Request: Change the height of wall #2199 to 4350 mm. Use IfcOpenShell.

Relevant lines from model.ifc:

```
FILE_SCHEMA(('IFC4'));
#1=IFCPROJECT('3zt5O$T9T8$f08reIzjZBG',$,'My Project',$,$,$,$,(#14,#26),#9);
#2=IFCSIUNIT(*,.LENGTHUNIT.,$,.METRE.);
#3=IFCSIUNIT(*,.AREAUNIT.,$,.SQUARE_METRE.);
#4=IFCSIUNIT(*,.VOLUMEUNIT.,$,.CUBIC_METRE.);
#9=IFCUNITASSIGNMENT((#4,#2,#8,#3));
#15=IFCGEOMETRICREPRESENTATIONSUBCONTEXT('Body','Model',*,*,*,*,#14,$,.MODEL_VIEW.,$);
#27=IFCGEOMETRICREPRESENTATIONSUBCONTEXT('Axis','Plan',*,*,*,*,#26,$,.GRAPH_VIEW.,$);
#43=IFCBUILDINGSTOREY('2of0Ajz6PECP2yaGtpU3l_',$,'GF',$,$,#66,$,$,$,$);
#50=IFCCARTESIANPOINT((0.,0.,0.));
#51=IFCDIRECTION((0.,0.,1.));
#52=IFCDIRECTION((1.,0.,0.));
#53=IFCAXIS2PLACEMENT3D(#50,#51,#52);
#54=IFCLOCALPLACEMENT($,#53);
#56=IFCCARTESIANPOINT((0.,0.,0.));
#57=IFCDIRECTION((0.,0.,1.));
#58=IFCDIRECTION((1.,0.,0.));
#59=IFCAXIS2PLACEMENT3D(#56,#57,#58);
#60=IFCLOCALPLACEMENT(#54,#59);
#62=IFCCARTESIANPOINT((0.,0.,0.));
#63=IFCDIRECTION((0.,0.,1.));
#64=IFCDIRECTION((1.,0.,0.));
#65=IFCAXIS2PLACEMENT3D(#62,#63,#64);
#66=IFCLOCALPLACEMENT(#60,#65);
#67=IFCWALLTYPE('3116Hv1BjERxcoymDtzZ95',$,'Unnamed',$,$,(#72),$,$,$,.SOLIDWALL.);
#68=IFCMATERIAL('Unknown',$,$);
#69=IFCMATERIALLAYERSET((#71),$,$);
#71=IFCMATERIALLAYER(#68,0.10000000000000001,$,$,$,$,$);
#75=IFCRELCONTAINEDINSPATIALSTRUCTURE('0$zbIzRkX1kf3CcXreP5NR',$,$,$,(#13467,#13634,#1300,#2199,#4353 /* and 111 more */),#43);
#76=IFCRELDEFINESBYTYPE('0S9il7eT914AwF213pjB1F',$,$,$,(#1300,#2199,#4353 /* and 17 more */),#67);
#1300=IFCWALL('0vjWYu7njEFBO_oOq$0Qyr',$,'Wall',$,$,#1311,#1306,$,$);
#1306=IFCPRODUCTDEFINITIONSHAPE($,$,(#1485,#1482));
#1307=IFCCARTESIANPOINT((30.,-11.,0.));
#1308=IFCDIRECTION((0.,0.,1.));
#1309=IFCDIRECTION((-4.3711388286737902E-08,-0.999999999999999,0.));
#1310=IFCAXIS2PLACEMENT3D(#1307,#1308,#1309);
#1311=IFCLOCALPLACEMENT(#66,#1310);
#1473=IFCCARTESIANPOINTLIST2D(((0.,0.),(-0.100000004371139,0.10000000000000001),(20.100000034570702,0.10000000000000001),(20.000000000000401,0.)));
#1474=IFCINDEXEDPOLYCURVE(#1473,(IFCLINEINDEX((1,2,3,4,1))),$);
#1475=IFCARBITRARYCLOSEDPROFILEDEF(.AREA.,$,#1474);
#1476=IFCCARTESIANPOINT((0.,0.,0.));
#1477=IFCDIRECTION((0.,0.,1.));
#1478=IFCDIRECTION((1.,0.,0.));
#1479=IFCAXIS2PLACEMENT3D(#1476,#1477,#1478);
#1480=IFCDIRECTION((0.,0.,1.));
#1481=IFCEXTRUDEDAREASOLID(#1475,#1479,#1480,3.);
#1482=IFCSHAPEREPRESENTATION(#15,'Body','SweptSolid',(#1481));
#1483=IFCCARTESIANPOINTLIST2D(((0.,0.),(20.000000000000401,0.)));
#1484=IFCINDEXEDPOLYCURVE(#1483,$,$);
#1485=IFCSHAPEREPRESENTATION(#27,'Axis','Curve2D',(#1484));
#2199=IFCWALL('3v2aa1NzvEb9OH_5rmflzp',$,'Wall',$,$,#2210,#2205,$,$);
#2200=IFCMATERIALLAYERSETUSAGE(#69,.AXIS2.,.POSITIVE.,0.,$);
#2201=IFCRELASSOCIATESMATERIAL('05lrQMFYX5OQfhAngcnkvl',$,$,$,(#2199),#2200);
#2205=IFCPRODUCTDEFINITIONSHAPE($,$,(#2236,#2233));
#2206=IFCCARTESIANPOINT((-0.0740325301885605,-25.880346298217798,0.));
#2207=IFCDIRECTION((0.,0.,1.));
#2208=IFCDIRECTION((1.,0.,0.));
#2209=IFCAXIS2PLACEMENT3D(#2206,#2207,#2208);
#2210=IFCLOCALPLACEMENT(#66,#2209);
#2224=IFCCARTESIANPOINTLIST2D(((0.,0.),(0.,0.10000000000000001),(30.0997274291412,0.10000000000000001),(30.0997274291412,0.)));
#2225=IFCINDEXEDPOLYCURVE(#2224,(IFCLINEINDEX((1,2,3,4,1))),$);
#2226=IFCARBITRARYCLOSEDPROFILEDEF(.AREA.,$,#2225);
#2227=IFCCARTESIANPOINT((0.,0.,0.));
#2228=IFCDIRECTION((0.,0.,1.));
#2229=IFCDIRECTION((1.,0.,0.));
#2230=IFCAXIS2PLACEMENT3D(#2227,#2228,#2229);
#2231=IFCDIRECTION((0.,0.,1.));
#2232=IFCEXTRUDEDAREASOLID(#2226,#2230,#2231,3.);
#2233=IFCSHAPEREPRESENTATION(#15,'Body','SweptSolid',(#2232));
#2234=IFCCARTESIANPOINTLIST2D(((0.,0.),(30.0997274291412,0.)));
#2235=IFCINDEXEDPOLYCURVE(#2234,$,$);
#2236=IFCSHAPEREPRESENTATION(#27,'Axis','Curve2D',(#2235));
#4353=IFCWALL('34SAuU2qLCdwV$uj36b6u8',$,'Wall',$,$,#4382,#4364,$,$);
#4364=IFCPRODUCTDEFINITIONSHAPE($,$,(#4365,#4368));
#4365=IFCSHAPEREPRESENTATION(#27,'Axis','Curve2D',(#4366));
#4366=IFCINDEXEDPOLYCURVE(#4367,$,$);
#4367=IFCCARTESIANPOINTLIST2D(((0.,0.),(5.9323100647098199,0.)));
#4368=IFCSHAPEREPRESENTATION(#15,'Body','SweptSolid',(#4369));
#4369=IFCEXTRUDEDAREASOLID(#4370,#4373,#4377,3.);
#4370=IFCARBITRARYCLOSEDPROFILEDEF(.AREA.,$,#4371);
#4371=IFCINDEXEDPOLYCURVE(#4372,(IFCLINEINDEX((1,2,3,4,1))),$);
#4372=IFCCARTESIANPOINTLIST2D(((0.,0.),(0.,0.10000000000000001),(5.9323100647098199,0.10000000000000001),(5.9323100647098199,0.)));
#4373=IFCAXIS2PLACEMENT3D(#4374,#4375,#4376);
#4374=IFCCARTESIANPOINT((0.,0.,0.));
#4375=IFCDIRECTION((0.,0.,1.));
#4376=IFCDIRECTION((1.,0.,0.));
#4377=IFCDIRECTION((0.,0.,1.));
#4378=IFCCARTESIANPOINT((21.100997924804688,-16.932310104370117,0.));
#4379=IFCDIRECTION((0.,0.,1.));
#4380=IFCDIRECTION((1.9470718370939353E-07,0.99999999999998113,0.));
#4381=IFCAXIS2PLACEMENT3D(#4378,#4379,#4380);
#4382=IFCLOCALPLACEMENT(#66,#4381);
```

```python
import ifcopenshell
import ifcopenshell.geom
import ifcopenshell.util.representation
import ifcopenshell.util.shape
import ifcopenshell.util.unit

model = ifcopenshell.open("model.ifc")
unit_scale = ifcopenshell.util.unit.calculate_unit_scale(model)
settings = ifcopenshell.geom.settings()


def volume(element):
    """Net volume in cubic metres, openings subtracted."""
    shape = ifcopenshell.geom.create_shape(settings, element)
    return ifcopenshell.util.shape.get_volume(shape.geometry)


wall = model.by_id(2199)
before = volume(wall)

body = ifcopenshell.util.representation.get_representation(wall, "Model", "Body")
solid = body.Items[0]
old_height = solid.Depth
solid.Depth = 4.35 / unit_scale
after = volume(wall)

print(f"height {old_height:g} -> {solid.Depth:g}, volume {before:.3f} -> {after:.3f} m3")

model.write("model_edited.ifc")
```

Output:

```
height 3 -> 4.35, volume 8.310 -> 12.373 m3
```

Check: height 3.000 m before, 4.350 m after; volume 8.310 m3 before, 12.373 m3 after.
